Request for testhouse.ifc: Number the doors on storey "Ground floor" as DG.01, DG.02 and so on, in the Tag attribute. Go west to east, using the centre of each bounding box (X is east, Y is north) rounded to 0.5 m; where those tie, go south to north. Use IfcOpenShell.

First a look at what the model holds.

```python
import ifcopenshell
import ifcopenshell.util.element
import ifcopenshell.util.placement

model = ifcopenshell.open("testhouse.ifc")
print(model.schema)
storey = next(s for s in model.by_type("IfcBuildingStorey") if s.Name == "Ground floor")
doors = [e for e in ifcopenshell.util.element.get_decomposition(storey) if e.is_a("IfcDoor")]
for e in sorted(doors, key=lambda e: e.id()):
    origin = ifcopenshell.util.placement.get_local_placement(e.ObjectPlacement)[:3, 3]
    print(e.id(), e.Tag, e.Name, origin.round(2) + 0.0, sep=" | ")
```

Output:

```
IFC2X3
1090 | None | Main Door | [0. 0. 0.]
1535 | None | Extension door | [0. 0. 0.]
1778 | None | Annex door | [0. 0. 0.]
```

```python
import ifcopenshell
import ifcopenshell.geom
import ifcopenshell.util.element
import ifcopenshell.util.shape

model = ifcopenshell.open("testhouse.ifc")
settings = ifcopenshell.geom.settings()
settings.set("use-world-coords", True)


def centre(element):
    shape = ifcopenshell.geom.create_shape(settings, element)
    return ifcopenshell.util.shape.get_bbox_centroid(shape.geometry)


storey = next(s for s in model.by_type("IfcBuildingStorey") if s.Name == "Ground floor")
doors = [e for e in ifcopenshell.util.element.get_decomposition(storey) if e.is_a("IfcDoor")]

# Insertion points can sit at a corner or the storey origin, so sort by the geometry (in metres).
centres = {e: centre(e) for e in doors}
doors.sort(key=lambda e: (round(centres[e][0] / 0.5), centres[e][1]))

for i, e in enumerate(doors, start=1):
    number = f"DG.{i:02d}"
    e.Tag = number
    print(e.id(), number)

model.write("testhouse_updated.ifc")
```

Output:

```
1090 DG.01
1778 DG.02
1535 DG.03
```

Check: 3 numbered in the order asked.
